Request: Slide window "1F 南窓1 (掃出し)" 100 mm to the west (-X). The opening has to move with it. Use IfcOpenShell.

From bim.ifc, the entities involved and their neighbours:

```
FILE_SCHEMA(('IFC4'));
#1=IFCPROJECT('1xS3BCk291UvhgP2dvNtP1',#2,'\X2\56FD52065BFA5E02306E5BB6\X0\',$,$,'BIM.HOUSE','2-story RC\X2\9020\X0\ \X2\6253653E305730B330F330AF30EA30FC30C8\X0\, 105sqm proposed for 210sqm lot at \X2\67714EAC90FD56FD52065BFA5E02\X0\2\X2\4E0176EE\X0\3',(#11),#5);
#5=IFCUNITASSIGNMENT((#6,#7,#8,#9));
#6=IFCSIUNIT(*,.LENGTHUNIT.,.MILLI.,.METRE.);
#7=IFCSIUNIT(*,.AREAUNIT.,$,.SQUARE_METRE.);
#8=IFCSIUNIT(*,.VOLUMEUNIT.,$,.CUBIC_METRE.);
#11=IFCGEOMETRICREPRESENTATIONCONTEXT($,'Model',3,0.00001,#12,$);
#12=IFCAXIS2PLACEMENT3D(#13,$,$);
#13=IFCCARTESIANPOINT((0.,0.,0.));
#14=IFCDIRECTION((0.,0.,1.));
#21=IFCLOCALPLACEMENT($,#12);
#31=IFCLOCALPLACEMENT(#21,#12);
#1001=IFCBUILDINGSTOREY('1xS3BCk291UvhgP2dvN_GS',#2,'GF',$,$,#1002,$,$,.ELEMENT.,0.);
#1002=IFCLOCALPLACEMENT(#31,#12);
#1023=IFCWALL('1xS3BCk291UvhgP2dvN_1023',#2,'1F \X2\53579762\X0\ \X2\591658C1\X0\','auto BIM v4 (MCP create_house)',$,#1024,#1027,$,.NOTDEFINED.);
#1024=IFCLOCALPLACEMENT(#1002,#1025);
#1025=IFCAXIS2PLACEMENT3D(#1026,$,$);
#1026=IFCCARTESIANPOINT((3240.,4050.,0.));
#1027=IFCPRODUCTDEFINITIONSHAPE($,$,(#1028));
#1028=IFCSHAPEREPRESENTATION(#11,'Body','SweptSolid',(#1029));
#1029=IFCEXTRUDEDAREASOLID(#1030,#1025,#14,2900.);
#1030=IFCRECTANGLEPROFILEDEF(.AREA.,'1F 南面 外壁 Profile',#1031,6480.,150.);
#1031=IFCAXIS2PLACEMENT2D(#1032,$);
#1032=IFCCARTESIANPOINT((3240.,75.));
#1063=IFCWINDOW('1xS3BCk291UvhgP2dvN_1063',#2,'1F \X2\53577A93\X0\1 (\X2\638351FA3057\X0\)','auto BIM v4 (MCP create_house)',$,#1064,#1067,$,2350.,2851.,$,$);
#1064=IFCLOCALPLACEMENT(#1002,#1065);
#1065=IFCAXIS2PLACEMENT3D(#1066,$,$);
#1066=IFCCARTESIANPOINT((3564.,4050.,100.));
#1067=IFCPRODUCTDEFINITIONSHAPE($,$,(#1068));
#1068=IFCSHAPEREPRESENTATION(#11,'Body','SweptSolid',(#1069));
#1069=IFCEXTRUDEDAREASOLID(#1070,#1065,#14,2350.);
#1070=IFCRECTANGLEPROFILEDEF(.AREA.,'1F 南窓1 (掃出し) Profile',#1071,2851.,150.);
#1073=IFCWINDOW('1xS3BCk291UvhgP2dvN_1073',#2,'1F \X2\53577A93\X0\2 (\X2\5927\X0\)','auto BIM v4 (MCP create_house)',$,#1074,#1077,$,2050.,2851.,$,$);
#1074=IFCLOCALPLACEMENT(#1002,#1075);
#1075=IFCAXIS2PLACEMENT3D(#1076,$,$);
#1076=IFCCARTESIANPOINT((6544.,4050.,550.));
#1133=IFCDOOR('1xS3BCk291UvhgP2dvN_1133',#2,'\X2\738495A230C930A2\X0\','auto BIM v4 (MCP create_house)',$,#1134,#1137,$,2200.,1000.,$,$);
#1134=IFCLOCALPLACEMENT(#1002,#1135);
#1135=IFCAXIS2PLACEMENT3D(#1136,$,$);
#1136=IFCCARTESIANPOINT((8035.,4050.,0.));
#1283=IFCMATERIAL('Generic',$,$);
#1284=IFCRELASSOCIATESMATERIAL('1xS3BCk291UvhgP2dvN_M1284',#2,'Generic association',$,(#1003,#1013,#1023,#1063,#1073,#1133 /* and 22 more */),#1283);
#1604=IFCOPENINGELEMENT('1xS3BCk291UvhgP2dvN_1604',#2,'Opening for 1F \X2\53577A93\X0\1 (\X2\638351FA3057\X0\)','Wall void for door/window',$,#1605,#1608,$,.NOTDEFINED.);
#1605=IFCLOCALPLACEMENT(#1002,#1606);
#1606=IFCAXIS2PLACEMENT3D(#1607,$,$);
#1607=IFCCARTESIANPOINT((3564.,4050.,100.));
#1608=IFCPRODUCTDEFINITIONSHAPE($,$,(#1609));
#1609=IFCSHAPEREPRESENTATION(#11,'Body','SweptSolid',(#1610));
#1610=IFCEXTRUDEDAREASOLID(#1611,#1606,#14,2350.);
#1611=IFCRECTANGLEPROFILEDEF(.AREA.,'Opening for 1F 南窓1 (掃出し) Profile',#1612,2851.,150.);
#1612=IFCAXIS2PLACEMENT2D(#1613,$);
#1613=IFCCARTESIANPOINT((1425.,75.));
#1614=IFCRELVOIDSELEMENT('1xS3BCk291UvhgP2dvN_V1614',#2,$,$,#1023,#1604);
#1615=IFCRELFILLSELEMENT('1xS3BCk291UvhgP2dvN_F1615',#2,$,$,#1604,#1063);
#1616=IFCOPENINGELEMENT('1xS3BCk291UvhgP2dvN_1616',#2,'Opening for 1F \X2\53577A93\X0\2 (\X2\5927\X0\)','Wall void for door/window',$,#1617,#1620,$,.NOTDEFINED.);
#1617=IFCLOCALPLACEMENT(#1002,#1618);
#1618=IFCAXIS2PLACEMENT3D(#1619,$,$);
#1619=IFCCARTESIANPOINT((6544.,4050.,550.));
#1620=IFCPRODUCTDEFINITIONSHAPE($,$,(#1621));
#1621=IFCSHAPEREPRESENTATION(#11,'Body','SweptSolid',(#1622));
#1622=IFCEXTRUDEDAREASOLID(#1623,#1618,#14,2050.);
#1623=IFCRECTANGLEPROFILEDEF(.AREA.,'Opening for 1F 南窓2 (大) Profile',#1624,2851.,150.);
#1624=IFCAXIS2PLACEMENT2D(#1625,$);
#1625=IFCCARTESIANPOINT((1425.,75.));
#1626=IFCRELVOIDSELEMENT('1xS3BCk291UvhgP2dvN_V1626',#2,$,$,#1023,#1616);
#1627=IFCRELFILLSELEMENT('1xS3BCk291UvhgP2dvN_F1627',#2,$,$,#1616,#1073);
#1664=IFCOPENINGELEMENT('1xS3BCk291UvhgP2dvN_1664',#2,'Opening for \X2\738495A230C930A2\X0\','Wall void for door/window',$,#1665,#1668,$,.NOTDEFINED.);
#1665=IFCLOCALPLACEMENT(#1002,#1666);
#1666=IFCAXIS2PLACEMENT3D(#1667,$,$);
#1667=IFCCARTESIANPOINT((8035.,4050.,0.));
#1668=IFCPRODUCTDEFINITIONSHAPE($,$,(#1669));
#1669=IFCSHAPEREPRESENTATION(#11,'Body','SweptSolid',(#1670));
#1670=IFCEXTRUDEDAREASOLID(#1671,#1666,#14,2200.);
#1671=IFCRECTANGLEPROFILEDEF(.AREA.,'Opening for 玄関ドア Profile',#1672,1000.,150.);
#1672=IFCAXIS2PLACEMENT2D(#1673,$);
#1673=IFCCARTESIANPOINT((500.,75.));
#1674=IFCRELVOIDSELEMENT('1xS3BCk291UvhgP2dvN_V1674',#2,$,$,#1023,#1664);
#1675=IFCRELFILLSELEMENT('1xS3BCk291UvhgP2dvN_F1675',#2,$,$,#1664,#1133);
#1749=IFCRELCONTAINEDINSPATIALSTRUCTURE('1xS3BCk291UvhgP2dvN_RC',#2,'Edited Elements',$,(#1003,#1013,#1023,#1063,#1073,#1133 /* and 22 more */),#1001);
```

```python
import ifcopenshell
import ifcopenshell.api.geometry
import ifcopenshell.util.placement
import ifcopenshell.util.unit

model = ifcopenshell.open("bim.ifc")
unit_scale = ifcopenshell.util.unit.calculate_unit_scale(model)

window = model.by_id(1063)
opening = window.FillsVoids[0].RelatingOpeningElement
wall = opening.VoidsElements[0].RelatingBuildingElement

wall_matrix = ifcopenshell.util.placement.get_local_placement(wall.ObjectPlacement)
shift = wall_matrix[:3, 0] * -0.1 / unit_scale
before = ifcopenshell.util.placement.get_local_placement(window.ObjectPlacement)[:3, 3].copy()

# The window is not placed relative to its opening, so move both.
for product in (opening, window):
    matrix = ifcopenshell.util.placement.get_local_placement(product.ObjectPlacement)
    matrix[:3, 3] += shift
    ifcopenshell.api.geometry.edit_object_placement(model, product=product, matrix=matrix, is_si=False)

after = ifcopenshell.util.placement.get_local_placement(window.ObjectPlacement)[:3, 3]
print("window moved by", (after - before).round(3) + 0.0)

model.write("bim_updated.ifc")
```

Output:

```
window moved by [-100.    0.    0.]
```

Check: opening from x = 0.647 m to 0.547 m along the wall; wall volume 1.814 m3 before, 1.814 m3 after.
